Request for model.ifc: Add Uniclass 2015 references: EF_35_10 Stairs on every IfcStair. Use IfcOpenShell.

First a look at what the model holds.

```python
import ifcopenshell

model = ifcopenshell.open("model.ifc")
print(model.schema)
print("classifications:", [c.Name for c in model.by_type("IfcClassification")])
for ifc_class in ("IfcDoor", "IfcRoof", "IfcStair", "IfcWall", "IfcWindow"):
    print(ifc_class, len(model.by_type(ifc_class)))
```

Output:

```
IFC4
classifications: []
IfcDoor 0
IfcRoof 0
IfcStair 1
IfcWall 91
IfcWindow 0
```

```python
import ifcopenshell
import ifcopenshell.api.classification

model = ifcopenshell.open("model.ifc")

system = ifcopenshell.api.classification.add_classification(model, classification="Uniclass 2015")

codes = {
    "IfcStair": ("EF_35_10", "Stairs"),
}
for ifc_class, (code, name) in codes.items():
    products = model.by_type(ifc_class)
    ifcopenshell.api.classification.add_reference(
        model, products=products, classification=system, identification=code, name=name
    )
    print(code, len(products))

model.write("model_edited.ifc")
```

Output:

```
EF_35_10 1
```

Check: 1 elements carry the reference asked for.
